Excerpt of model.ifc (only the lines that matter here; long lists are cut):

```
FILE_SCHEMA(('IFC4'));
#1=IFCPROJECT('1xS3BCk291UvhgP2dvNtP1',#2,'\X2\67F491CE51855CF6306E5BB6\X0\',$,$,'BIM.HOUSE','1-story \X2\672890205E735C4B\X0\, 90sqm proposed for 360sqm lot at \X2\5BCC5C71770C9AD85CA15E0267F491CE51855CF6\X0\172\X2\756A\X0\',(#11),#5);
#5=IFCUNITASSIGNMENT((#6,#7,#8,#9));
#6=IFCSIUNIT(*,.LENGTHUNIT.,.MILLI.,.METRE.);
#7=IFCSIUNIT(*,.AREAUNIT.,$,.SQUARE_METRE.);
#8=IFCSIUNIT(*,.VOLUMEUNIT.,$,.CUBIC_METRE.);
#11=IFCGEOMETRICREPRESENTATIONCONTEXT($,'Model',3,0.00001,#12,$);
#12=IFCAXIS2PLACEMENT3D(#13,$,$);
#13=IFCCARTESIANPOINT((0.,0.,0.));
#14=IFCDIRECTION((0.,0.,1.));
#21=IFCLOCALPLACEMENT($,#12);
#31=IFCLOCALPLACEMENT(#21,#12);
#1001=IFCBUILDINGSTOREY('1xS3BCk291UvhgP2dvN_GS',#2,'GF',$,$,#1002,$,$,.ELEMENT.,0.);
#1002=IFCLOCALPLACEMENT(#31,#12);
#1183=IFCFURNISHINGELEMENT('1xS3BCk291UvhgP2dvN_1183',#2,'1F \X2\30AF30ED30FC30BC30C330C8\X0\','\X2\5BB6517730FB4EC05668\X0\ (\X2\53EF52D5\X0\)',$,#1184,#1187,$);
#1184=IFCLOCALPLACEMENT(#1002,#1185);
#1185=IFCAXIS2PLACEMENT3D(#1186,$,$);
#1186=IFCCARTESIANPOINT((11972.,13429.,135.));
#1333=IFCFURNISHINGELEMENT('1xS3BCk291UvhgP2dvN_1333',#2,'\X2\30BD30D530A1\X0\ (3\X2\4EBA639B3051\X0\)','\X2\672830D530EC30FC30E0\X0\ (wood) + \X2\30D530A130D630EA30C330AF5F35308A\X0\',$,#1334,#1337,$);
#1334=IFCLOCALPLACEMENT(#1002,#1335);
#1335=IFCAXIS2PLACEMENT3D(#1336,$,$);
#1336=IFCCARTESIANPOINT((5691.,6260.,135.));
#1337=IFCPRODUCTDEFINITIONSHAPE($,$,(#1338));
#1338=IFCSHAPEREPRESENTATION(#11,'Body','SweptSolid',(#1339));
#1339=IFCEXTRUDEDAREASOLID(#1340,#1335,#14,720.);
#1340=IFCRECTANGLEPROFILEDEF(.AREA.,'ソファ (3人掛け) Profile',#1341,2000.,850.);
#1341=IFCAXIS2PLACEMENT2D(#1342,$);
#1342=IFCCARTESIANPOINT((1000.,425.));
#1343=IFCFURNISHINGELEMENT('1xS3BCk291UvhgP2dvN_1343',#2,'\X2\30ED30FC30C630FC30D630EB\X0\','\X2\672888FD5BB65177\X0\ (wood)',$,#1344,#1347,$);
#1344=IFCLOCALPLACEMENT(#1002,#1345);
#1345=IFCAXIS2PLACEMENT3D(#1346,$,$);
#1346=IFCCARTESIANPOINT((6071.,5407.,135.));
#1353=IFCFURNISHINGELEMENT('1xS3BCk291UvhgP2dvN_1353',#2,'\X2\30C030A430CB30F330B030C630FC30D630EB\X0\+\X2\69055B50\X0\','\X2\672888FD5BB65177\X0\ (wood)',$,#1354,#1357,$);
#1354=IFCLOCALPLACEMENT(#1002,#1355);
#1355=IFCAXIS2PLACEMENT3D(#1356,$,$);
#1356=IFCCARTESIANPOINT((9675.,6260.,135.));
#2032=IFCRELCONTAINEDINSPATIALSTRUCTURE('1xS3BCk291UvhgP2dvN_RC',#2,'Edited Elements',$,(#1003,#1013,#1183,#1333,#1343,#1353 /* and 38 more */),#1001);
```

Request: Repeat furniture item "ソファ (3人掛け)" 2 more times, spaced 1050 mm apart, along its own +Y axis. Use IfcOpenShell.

```python
import ifcopenshell
import ifcopenshell.api.geometry
import ifcopenshell.api.root
import ifcopenshell.util.element
import ifcopenshell.util.placement

model = ifcopenshell.open("model.ifc")


def reuse_history(source, copy):
    """copy_class also copies each property set's owner history, people and application; keep the originals."""
    for rel in copy.IsDefinedBy:
        if rel.is_a("IfcRelDefinesByProperties") and (history := rel.RelatingPropertyDefinition.OwnerHistory):
            rel.RelatingPropertyDefinition.OwnerHistory = source.OwnerHistory
            ifcopenshell.util.element.remove_deep2(model, history)


source = model.by_guid("1xS3BCk291UvhgP2dvN_1333")
base = ifcopenshell.util.placement.get_local_placement(source.ObjectPlacement)
step = base[:3, 1] * 1050.0

for i in range(1, 3):
    copy = ifcopenshell.api.root.copy_class(model, product=source)
    copy.Representation = ifcopenshell.util.element.copy_deep(
        model, source.Representation, exclude=["IfcGeometricRepresentationContext", "IfcRepresentationMap"]
    )
    reuse_history(source, copy)
    matrix = base.copy()
    matrix[:3, 3] += i * step
    print("added at", matrix[:3, 3].round(3) + 0.0)
    ifcopenshell.api.geometry.edit_object_placement(model, product=copy, matrix=matrix, is_si=False)

model.write("model-out.ifc")
```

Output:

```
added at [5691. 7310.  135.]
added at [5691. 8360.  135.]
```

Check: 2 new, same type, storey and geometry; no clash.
